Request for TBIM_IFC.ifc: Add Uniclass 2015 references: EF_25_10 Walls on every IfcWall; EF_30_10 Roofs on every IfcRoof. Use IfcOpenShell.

First a look at what the model holds.

```python
import ifcopenshell

model = ifcopenshell.open("TBIM_IFC.ifc")
print(model.schema)
print("classifications:", [c.Name for c in model.by_type("IfcClassification")])
for ifc_class in ("IfcDoor", "IfcRoof", "IfcStair", "IfcWall", "IfcWindow"):
    print(ifc_class, len(model.by_type(ifc_class)))
```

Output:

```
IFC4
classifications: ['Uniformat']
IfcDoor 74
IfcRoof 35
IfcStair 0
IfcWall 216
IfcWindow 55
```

```python
import ifcopenshell
import ifcopenshell.api.classification

model = ifcopenshell.open("TBIM_IFC.ifc")

system = ifcopenshell.api.classification.add_classification(model, classification="Uniclass 2015")

codes = {
    "IfcWall": ("EF_25_10", "Walls"),
    "IfcRoof": ("EF_30_10", "Roofs"),
}
for ifc_class, (code, name) in codes.items():
    products = model.by_type(ifc_class)
    ifcopenshell.api.classification.add_reference(
        model, products=products, classification=system, identification=code, name=name
    )
    print(code, len(products))

model.write("TBIM_IFC_updated.ifc")
```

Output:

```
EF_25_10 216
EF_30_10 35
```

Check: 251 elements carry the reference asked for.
